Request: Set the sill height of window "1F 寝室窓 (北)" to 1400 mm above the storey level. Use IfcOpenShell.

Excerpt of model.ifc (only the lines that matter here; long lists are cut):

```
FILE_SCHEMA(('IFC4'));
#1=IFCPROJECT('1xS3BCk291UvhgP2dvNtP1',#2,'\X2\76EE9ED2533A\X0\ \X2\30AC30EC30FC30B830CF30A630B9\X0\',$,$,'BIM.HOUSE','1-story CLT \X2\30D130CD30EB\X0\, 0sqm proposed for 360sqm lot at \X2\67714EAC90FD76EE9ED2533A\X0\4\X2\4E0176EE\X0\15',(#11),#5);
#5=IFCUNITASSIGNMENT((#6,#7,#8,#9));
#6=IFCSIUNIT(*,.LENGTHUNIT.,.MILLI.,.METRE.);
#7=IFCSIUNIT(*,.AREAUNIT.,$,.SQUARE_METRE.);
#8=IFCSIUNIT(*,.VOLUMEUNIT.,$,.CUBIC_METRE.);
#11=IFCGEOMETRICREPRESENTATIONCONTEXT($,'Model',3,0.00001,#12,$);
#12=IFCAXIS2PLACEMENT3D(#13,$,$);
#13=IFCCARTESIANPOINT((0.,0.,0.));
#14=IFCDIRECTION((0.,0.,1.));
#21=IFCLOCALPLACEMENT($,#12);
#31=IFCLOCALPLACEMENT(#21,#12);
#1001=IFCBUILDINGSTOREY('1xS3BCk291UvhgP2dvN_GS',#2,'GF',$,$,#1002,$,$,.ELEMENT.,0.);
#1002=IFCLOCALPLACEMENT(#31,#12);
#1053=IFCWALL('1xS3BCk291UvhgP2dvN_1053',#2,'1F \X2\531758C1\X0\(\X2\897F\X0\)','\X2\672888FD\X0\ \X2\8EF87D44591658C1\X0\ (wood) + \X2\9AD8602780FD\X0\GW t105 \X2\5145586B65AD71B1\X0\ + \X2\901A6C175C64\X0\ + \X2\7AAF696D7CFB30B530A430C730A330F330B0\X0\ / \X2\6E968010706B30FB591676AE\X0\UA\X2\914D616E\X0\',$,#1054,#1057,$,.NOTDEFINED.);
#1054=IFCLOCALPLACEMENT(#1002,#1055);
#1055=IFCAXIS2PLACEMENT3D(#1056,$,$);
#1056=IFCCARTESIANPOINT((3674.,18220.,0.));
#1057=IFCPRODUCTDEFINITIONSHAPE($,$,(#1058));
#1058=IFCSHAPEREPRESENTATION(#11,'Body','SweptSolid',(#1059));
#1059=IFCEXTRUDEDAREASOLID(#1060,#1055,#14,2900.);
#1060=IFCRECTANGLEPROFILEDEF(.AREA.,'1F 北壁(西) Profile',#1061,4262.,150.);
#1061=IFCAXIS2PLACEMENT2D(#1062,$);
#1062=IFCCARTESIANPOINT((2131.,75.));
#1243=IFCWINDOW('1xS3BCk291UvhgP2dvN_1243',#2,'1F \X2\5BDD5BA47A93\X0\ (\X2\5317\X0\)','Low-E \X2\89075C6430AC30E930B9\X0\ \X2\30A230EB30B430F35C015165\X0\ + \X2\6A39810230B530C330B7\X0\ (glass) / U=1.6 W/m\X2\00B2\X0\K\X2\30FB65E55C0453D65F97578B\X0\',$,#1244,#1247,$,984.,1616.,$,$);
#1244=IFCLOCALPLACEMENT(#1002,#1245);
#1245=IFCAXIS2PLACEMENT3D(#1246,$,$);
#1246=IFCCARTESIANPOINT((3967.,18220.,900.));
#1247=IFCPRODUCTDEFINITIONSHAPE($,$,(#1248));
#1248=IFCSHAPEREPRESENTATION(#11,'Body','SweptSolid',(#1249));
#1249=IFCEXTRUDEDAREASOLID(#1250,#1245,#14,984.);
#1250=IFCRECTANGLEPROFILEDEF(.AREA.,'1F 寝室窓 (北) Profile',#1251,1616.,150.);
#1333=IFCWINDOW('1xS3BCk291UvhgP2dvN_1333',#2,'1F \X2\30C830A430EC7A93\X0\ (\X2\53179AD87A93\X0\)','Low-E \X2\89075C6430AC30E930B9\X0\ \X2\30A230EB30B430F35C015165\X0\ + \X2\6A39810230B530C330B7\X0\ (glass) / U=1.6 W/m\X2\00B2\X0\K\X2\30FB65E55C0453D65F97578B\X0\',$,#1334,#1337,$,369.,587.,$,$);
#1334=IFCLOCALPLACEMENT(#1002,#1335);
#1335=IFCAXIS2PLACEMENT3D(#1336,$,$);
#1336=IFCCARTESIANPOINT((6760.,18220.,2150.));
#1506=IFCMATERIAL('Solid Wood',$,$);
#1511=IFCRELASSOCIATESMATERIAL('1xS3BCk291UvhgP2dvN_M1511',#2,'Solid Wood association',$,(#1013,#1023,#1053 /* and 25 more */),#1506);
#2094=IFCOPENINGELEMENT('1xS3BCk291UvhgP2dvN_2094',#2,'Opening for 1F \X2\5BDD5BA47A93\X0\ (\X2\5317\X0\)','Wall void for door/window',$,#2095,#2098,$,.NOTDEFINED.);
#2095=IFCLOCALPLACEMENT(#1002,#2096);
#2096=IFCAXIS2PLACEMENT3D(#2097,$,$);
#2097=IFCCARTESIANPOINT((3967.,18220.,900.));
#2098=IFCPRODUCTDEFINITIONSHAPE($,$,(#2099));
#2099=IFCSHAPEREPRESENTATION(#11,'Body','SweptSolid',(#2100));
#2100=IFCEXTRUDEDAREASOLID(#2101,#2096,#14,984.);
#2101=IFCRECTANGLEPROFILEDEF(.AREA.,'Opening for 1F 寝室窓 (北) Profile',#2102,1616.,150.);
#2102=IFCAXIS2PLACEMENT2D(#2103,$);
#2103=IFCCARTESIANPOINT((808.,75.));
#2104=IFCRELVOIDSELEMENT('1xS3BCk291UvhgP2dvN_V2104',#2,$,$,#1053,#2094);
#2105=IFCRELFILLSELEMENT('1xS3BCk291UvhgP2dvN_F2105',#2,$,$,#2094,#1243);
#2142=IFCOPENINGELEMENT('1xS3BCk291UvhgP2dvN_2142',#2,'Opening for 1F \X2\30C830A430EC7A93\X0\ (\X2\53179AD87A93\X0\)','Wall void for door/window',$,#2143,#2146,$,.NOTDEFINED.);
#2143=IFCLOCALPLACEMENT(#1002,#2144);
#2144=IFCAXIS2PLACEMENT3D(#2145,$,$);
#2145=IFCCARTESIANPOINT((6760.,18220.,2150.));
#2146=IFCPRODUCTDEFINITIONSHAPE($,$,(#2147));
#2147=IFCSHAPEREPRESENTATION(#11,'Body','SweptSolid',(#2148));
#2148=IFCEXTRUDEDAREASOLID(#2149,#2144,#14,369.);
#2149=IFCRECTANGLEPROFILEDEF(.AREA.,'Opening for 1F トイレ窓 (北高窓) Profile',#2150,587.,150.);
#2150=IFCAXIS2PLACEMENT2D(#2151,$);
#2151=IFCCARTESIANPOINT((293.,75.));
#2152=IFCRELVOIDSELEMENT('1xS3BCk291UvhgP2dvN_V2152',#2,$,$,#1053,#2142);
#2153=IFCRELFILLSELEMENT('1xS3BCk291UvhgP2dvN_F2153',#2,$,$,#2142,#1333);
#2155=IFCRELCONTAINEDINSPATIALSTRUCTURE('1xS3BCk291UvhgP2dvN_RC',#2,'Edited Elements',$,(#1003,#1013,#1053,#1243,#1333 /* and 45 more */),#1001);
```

```python
import numpy as np
import ifcopenshell
import ifcopenshell.api.geometry
import ifcopenshell.geom
import ifcopenshell.util.element
import ifcopenshell.util.placement
import ifcopenshell.util.shape
import ifcopenshell.util.unit

model = ifcopenshell.open("model.ifc")
unit_scale = ifcopenshell.util.unit.calculate_unit_scale(model)

window = model.by_guid("1xS3BCk291UvhgP2dvN_1243")
opening = window.FillsVoids[0].RelatingOpeningElement
storey = ifcopenshell.util.element.get_container(window, ifc_class="IfcBuildingStorey")
level = ifcopenshell.util.placement.get_local_placement(storey.ObjectPlacement)[2, 3]

# The opening's origin need not be at the sill, so measure its lowest point.
shape = ifcopenshell.geom.create_shape(ifcopenshell.geom.settings(), opening)
bottom = ifcopenshell.util.shape.get_shape_bottom_elevation(shape, shape.geometry) / unit_scale
dz = level + 1.4 / unit_scale - bottom

shift = np.array([0.0, 0.0, dz])
# The window is not placed relative to its opening, so move both.
for product in (opening, window):
    matrix = ifcopenshell.util.placement.get_local_placement(product.ObjectPlacement)
    matrix[:3, 3] += shift
    ifcopenshell.api.geometry.edit_object_placement(model, product=product, matrix=matrix, is_si=False)

print(f"moved by {dz * unit_scale:+.3f} m")

model.write("model-out.ifc")
```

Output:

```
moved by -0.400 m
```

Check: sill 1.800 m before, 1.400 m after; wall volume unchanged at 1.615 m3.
